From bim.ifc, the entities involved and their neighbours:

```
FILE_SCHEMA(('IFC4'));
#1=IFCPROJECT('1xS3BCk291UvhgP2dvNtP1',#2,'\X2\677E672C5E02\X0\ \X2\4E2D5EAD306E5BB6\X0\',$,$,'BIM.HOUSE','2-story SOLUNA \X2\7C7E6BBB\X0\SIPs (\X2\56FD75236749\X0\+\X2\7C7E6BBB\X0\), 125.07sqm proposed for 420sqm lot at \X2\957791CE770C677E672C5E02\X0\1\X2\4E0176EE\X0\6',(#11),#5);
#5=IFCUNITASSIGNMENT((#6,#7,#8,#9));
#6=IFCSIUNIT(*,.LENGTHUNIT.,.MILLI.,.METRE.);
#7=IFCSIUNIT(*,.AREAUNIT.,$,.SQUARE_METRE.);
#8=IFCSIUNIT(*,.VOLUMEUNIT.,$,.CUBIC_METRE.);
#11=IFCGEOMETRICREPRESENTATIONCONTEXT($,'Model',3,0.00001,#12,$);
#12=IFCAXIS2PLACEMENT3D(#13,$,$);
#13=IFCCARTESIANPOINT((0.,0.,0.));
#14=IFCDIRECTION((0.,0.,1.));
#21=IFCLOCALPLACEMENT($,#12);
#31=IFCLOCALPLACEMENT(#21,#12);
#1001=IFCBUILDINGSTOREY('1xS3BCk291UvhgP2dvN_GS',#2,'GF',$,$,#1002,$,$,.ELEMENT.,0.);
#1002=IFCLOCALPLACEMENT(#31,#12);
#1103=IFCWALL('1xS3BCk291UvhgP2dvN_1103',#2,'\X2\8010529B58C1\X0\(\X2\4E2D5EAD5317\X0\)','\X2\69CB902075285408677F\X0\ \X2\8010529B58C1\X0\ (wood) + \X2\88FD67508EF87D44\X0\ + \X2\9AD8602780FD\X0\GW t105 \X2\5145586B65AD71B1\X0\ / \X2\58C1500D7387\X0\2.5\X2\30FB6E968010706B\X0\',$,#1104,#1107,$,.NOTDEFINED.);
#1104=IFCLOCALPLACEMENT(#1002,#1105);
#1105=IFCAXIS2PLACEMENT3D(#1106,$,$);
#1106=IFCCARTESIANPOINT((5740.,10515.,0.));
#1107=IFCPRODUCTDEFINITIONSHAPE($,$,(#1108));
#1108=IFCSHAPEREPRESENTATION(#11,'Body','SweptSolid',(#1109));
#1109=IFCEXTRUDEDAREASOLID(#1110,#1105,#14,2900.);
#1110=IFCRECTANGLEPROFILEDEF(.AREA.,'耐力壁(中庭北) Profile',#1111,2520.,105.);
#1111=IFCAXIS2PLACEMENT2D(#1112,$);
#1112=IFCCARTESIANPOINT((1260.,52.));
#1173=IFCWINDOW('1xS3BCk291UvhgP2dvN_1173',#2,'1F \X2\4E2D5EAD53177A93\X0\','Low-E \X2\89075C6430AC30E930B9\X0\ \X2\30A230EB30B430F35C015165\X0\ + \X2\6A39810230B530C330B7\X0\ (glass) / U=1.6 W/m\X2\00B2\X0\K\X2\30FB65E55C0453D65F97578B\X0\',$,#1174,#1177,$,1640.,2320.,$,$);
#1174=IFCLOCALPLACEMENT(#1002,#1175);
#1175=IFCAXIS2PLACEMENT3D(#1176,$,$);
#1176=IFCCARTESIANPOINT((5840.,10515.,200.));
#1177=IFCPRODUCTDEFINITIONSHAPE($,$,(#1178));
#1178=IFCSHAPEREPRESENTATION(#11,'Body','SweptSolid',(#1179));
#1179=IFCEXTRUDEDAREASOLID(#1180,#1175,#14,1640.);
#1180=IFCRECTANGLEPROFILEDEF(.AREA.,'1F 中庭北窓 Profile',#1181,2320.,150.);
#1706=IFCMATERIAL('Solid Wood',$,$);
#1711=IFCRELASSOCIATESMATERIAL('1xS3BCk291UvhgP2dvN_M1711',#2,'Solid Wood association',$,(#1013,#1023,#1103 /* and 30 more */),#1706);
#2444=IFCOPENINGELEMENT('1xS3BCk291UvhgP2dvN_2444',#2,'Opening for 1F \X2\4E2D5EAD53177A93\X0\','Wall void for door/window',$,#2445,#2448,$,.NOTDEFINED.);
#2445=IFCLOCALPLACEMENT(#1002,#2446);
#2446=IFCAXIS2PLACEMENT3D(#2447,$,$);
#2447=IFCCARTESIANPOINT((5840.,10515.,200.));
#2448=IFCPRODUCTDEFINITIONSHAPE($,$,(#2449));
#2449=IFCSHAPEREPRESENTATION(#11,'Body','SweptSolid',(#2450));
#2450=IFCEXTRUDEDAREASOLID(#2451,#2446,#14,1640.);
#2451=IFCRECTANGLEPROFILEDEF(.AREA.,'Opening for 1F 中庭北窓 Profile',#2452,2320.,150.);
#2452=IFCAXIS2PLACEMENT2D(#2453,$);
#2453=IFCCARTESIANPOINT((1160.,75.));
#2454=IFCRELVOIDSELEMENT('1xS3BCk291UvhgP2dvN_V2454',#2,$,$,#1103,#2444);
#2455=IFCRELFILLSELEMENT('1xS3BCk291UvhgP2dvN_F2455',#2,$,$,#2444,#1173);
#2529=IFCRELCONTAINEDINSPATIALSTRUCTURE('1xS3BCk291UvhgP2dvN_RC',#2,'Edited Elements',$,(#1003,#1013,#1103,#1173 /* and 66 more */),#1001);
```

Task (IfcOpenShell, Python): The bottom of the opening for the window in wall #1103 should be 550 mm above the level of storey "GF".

```python
import numpy as np
import ifcopenshell
import ifcopenshell.api.geometry
import ifcopenshell.geom
import ifcopenshell.util.element
import ifcopenshell.util.placement
import ifcopenshell.util.shape
import ifcopenshell.util.unit

model = ifcopenshell.open("bim.ifc")
unit_scale = ifcopenshell.util.unit.calculate_unit_scale(model)

window = model.by_guid("1xS3BCk291UvhgP2dvN_1173")
opening = window.FillsVoids[0].RelatingOpeningElement
storey = ifcopenshell.util.element.get_container(window, ifc_class="IfcBuildingStorey")
level = ifcopenshell.util.placement.get_local_placement(storey.ObjectPlacement)[2, 3]

# The opening's origin need not be at the sill, so measure its lowest point.
shape = ifcopenshell.geom.create_shape(ifcopenshell.geom.settings(), opening)
bottom = ifcopenshell.util.shape.get_shape_bottom_elevation(shape, shape.geometry) / unit_scale
dz = level + 0.55 / unit_scale - bottom

shift = np.array([0.0, 0.0, dz])
# The window is not placed relative to its opening, so move both.
for product in (opening, window):
    matrix = ifcopenshell.util.placement.get_local_placement(product.ObjectPlacement)
    matrix[:3, 3] += shift
    ifcopenshell.api.geometry.edit_object_placement(model, product=product, matrix=matrix, is_si=False)

print(f"moved by {dz * unit_scale:+.3f} m")

model.write("bim_updated.ifc")
```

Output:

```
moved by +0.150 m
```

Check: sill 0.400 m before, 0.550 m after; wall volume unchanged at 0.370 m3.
